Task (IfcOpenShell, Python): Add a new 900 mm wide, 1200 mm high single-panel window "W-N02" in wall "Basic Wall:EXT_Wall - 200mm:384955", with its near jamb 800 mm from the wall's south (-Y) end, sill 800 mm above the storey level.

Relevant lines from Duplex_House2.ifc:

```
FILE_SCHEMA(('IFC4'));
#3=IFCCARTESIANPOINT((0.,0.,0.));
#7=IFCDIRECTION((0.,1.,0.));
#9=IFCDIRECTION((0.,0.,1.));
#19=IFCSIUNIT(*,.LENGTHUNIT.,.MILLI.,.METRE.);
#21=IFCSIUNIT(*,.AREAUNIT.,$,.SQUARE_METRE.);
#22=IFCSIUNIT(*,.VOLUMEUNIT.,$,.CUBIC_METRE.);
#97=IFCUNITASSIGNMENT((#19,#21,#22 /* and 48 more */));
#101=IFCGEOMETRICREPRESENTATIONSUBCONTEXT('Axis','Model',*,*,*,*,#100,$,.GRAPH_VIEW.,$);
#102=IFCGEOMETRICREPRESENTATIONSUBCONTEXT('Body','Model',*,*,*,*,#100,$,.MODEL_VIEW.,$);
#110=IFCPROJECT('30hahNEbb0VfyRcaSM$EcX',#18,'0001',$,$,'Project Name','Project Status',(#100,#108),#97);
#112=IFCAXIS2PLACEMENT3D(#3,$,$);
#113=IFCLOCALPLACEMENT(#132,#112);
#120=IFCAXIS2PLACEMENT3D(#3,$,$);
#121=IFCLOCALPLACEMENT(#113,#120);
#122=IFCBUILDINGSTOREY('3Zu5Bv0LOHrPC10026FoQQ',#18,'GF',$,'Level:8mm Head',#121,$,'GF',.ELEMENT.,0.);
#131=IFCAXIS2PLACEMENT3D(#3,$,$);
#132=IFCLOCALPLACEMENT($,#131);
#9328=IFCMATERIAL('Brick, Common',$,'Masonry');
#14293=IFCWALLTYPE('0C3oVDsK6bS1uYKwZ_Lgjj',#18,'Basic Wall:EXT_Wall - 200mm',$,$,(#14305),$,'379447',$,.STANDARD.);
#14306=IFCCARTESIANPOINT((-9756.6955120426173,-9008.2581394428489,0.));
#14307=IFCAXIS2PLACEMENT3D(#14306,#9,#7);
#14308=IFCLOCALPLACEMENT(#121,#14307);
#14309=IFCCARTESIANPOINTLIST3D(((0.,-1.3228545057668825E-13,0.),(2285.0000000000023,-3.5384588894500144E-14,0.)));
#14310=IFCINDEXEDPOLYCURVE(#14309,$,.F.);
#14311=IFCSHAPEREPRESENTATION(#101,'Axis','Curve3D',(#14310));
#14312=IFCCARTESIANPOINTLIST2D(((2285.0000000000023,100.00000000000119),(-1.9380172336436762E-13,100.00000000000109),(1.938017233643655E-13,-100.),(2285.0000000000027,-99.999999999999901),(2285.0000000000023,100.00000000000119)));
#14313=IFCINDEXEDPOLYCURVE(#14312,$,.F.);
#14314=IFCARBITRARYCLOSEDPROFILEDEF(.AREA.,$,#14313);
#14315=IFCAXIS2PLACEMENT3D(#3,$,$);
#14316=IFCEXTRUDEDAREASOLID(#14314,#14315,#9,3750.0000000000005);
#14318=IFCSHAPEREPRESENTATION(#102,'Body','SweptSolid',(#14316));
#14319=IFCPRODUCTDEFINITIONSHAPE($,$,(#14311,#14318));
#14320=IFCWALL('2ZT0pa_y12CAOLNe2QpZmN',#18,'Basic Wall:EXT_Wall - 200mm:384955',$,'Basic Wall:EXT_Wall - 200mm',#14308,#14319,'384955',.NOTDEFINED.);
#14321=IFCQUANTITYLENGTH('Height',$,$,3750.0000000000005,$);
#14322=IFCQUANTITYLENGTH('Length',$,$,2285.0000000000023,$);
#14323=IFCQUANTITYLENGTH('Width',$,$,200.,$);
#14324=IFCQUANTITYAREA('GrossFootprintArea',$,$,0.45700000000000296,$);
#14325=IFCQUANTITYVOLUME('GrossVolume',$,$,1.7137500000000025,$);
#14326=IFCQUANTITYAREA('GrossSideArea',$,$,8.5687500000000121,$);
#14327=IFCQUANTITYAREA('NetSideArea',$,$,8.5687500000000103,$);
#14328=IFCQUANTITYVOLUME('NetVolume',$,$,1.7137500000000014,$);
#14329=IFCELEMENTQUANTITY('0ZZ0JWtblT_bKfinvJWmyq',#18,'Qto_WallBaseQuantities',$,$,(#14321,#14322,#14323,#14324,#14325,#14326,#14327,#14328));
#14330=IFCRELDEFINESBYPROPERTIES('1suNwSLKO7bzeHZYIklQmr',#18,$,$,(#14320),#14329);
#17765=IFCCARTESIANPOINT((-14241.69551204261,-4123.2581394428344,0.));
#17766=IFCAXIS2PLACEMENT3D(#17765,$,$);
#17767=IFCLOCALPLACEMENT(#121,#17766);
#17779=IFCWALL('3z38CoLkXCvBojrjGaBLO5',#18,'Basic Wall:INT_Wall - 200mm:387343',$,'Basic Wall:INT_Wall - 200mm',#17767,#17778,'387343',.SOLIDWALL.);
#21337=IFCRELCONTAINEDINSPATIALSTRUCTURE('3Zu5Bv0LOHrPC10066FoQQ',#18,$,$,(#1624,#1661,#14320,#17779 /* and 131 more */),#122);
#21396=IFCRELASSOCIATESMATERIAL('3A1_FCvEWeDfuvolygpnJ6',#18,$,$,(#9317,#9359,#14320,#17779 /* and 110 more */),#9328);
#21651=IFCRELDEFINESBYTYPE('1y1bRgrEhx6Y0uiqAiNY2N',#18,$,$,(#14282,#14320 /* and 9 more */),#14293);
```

```python
import numpy as np
import ifcopenshell
import ifcopenshell.api.feature
import ifcopenshell.api.geometry
import ifcopenshell.api.pset
import ifcopenshell.api.root
import ifcopenshell.api.spatial
import ifcopenshell.geom
import ifcopenshell.util.element
import ifcopenshell.util.placement
import ifcopenshell.util.representation
import ifcopenshell.util.shape
import ifcopenshell.util.unit

model = ifcopenshell.open("Duplex_House2.ifc")
unit_scale = ifcopenshell.util.unit.calculate_unit_scale(model)
area_scale = ifcopenshell.util.unit.calculate_unit_scale(model, "AREAUNIT")
volume_scale = ifcopenshell.util.unit.calculate_unit_scale(model, "VOLUMEUNIT")
settings = ifcopenshell.geom.settings()


def volume(element):
    """Net volume in cubic metres, openings subtracted."""
    shape = ifcopenshell.geom.create_shape(settings, element)
    return ifcopenshell.util.shape.get_volume(shape.geometry)


wall = model.by_id(14320)
storey = ifcopenshell.util.element.get_container(wall, ifc_class="IfcBuildingStorey")
context = ifcopenshell.util.representation.get_context(model, "Model", "Body", "MODEL_VIEW")
before = volume(wall)

width, height, from_end, sill = 0.9, 1.2, 0.8, 0.8  # metres

# The wall runs along its own X axis, and the end named is its -X end.
wall_shape = ifcopenshell.geom.create_shape(settings, wall)
x, y, z = ifcopenshell.util.shape.get_vertices(wall_shape.geometry).T
start = x.min() + from_end
face, thickness = float(y.min()), float(y.max() - y.min())
wall_matrix = ifcopenshell.util.placement.get_local_placement(wall.ObjectPlacement)
level = ifcopenshell.util.placement.get_local_placement(storey.ObjectPlacement)[2, 3]


def in_wall(x, y):
    """Placement at x, y metres in the wall's axes, at sill height."""
    matrix = wall_matrix.copy()
    matrix[:, 3] = wall_matrix @ np.array([x / unit_scale, y / unit_scale, 0.0, 1.0])
    matrix[2, 3] = level + sill / unit_scale
    return matrix


# Opening: a box that overshoots both wall faces by 50 mm.
opening = ifcopenshell.api.root.create_entity(model, ifc_class="IfcOpeningElement", predefined_type="OPENING")
box = ifcopenshell.api.geometry.add_wall_representation(
    model, context=context, length=width, height=height, thickness=thickness + 0.1
)
ifcopenshell.api.geometry.assign_representation(model, product=opening, representation=box)
ifcopenshell.api.geometry.edit_object_placement(model, product=opening, matrix=in_wall(start, face - 0.05), is_si=False)
ifcopenshell.api.feature.add_feature(model, feature=opening, element=wall)

window = ifcopenshell.api.root.create_entity(model, ifc_class="IfcWindow", name="W-N02", predefined_type="WINDOW")
window.OverallWidth, window.OverallHeight = width / unit_scale, height / unit_scale
window.PartitioningType = "SINGLE_PANEL"
body = ifcopenshell.api.geometry.add_window_representation(
    model,
    context=context,
    overall_width=window.OverallWidth,
    overall_height=window.OverallHeight,
    partition_type="SINGLE_PANEL",
)
ifcopenshell.api.geometry.assign_representation(model, product=window, representation=body)
ifcopenshell.api.spatial.assign_container(model, products=[window], relating_structure=storey)
ifcopenshell.api.feature.add_filling(model, opening=opening, element=window)

# Centre the window in the wall's thickness.
ifcopenshell.api.geometry.edit_object_placement(model, product=window, matrix=in_wall(start, face), is_si=False)
window_shape = ifcopenshell.geom.create_shape(settings, window)
depth = ifcopenshell.util.shape.get_vertices(window_shape.geometry)[:, 1]
offset = face + thickness / 2 - (depth.min() + depth.max()) / 2
ifcopenshell.api.geometry.edit_object_placement(model, product=window, matrix=in_wall(start, offset), is_si=False)

after = volume(wall)

# Update the wall's stored quantities.
qto = model.by_id(ifcopenshell.util.element.get_pset(wall, "Qto_WallBaseQuantities", should_inherit=False)["id"])
ifcopenshell.api.pset.edit_qto(model, qto=qto, properties={
    "NetSideArea": after / thickness / area_scale,
    "NetVolume": after / volume_scale,
})

print(f"wall volume {before:.3f} -> {after:.3f} m3")

model.write("Duplex_House2_rev.ifc")
```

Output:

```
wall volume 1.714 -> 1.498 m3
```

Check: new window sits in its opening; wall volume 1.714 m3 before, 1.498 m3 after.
